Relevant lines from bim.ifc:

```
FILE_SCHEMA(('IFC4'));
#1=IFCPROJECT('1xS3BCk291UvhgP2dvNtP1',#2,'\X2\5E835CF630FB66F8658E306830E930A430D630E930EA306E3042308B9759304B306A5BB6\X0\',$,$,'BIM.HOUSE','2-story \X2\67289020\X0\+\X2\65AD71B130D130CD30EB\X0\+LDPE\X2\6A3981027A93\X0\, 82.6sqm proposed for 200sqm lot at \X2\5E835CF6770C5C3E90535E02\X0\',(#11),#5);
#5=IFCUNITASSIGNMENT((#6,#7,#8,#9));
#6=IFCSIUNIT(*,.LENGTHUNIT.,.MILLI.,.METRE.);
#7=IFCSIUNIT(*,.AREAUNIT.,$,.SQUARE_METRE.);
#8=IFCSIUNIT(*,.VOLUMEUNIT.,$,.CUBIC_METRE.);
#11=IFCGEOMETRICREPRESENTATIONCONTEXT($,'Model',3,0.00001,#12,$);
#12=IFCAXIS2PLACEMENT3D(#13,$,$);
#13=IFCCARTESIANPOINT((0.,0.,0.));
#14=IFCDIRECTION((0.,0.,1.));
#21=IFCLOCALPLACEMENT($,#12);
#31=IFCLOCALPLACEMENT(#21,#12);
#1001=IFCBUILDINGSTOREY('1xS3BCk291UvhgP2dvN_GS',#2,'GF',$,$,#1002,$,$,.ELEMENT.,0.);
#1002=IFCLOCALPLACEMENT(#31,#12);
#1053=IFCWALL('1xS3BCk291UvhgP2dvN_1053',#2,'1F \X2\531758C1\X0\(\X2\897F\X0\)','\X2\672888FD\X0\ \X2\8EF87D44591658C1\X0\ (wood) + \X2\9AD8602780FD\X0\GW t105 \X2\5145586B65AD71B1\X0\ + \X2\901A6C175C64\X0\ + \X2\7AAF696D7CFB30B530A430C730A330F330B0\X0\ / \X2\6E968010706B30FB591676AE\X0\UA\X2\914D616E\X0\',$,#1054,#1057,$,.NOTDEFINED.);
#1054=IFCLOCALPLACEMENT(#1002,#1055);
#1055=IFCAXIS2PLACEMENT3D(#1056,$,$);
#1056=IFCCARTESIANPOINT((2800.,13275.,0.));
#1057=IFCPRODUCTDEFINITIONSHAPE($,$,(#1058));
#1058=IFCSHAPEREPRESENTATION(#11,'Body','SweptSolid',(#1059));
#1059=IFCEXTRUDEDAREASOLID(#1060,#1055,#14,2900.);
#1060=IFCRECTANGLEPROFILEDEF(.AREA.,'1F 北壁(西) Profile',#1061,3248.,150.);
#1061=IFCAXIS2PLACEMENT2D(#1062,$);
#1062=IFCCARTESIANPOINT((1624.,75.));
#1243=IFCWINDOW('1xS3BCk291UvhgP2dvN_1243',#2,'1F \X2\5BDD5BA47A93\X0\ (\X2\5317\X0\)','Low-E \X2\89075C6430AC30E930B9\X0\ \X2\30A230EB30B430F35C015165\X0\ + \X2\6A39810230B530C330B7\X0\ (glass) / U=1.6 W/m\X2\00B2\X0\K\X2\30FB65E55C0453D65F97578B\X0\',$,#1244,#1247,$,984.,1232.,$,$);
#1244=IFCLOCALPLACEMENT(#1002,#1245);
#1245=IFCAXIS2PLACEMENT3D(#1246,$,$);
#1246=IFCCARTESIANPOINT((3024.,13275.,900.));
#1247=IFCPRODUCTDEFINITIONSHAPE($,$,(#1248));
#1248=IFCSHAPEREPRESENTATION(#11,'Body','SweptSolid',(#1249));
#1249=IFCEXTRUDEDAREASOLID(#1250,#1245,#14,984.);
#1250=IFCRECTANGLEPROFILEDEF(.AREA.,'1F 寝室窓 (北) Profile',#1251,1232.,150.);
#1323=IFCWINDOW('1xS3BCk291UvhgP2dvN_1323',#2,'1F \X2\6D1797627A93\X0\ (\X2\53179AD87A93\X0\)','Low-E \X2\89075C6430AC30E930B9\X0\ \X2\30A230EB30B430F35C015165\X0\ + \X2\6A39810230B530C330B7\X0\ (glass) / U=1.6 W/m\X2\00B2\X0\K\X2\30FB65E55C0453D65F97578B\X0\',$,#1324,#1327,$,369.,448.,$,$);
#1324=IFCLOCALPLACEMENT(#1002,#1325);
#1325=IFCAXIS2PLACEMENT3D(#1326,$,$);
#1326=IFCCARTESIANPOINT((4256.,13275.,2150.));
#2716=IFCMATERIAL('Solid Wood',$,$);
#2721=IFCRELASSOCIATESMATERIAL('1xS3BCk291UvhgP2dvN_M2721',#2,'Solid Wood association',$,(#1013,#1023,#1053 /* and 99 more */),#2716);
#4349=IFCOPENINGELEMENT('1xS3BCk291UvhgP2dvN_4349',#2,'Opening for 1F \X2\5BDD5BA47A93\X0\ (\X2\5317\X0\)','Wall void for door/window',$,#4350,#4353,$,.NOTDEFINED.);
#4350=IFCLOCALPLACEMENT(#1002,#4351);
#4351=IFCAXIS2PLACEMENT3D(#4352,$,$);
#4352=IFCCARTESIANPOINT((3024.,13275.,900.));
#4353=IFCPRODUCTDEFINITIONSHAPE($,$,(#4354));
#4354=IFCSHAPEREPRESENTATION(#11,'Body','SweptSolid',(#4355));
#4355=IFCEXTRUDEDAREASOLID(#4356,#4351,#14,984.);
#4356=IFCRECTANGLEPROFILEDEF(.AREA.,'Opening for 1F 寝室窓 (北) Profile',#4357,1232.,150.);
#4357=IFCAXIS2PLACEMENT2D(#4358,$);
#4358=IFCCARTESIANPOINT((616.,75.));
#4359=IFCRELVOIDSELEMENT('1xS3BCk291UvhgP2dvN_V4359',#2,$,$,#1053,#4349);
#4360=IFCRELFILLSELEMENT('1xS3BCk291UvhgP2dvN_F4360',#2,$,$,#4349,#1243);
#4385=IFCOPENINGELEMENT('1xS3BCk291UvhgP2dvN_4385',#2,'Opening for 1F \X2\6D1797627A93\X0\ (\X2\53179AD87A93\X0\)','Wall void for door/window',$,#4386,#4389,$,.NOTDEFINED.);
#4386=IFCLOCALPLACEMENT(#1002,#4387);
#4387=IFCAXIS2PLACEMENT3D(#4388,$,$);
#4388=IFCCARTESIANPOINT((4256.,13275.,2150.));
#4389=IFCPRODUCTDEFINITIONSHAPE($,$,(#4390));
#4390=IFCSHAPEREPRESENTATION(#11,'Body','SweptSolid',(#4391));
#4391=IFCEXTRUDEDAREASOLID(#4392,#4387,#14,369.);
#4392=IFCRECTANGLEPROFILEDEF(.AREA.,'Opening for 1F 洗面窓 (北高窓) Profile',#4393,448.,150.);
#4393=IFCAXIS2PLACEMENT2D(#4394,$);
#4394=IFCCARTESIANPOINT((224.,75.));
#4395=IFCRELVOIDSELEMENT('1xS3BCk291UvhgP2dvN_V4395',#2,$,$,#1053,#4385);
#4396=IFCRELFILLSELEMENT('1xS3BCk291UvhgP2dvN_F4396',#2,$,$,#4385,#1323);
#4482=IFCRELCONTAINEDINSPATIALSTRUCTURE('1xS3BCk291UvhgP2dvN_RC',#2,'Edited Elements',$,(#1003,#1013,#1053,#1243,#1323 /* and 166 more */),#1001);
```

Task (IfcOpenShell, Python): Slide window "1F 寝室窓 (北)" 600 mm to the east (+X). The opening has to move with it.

```python
import ifcopenshell
import ifcopenshell.api.geometry
import ifcopenshell.util.placement

model = ifcopenshell.open("bim.ifc")

window = model.by_id(1243)
opening = window.FillsVoids[0].RelatingOpeningElement
wall = opening.VoidsElements[0].RelatingBuildingElement

wall_matrix = ifcopenshell.util.placement.get_local_placement(wall.ObjectPlacement)
shift = wall_matrix[:3, 0] * 600.0
before = ifcopenshell.util.placement.get_local_placement(window.ObjectPlacement)[:3, 3].copy()

# The window is not placed relative to its opening, so move both.
for product in (opening, window):
    matrix = ifcopenshell.util.placement.get_local_placement(product.ObjectPlacement)
    matrix[:3, 3] += shift
    ifcopenshell.api.geometry.edit_object_placement(model, product=product, matrix=matrix, is_si=False)

after = ifcopenshell.util.placement.get_local_placement(window.ObjectPlacement)[:3, 3]
print("window moved by", (after - before).round(3) + 0.0)

model.write("bim_edited.ifc")
```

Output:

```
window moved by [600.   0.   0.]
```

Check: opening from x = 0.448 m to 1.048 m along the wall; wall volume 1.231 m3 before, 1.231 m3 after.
